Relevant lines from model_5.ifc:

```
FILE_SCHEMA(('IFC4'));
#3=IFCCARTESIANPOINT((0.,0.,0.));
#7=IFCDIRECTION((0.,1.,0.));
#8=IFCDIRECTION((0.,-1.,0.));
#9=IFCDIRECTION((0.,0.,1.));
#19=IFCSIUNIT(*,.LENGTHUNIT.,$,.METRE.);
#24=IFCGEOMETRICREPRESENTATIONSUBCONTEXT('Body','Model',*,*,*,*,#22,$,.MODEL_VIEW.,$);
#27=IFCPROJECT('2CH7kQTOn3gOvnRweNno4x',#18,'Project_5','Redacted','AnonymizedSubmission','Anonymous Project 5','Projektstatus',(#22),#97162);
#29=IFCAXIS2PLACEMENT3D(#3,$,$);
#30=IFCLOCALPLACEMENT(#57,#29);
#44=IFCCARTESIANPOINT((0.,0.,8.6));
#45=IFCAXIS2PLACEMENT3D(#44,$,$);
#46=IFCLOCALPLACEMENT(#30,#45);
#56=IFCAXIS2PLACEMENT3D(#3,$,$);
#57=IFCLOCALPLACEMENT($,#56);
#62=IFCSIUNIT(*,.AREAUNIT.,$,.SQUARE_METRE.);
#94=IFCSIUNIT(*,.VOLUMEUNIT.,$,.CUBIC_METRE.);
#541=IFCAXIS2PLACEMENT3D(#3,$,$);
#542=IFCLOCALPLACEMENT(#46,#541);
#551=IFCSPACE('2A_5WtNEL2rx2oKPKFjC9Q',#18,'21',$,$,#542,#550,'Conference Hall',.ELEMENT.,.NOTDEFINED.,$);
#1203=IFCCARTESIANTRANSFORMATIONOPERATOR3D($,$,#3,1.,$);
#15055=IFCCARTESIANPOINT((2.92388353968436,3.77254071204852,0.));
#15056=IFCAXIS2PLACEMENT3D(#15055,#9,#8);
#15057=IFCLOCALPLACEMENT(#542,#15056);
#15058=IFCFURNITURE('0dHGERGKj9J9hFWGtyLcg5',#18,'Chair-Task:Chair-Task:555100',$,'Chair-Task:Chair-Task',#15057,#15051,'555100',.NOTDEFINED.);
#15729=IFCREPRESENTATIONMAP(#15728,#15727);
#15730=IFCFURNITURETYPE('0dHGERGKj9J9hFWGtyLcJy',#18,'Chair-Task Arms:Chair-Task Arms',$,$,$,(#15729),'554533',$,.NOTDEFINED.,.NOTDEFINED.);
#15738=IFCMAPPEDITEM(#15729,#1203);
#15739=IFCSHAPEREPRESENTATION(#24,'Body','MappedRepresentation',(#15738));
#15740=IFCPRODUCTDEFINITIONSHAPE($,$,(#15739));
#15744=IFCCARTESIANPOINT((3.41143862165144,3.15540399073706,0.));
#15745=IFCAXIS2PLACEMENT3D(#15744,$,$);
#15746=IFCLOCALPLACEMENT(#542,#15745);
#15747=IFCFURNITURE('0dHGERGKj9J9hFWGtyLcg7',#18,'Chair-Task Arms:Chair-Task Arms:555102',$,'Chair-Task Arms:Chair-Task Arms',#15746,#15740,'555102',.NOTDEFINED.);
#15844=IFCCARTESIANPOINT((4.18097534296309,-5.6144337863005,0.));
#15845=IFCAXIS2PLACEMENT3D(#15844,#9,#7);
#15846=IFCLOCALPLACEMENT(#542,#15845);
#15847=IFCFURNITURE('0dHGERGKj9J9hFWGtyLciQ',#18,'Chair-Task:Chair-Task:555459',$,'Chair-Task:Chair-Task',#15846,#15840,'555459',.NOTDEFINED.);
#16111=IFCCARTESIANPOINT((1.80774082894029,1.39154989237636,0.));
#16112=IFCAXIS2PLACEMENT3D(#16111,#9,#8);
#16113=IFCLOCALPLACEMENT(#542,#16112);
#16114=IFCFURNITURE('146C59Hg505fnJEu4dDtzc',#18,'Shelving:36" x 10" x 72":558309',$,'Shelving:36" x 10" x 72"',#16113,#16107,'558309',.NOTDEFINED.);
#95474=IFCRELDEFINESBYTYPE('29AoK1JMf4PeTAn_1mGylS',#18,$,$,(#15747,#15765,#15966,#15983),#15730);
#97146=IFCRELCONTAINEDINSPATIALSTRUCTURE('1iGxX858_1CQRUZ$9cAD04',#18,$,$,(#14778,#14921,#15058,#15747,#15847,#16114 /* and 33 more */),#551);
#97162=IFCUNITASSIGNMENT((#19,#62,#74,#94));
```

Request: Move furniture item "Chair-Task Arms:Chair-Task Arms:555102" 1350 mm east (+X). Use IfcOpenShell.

```python
import ifcopenshell
import ifcopenshell.api.geometry
import ifcopenshell.util.placement
import ifcopenshell.util.unit

model = ifcopenshell.open("model_5.ifc")
unit_scale = ifcopenshell.util.unit.calculate_unit_scale(model)

item = model.by_guid("0dHGERGKj9J9hFWGtyLcg7")
matrix = ifcopenshell.util.placement.get_local_placement(item.ObjectPlacement)
matrix[0, 3] += 1.35 / unit_scale
ifcopenshell.api.geometry.edit_object_placement(model, product=item, matrix=matrix, is_si=False)

print(ifcopenshell.util.placement.get_local_placement(item.ObjectPlacement).round(3) + 0.0)

model.write("model_5_updated.ifc")
```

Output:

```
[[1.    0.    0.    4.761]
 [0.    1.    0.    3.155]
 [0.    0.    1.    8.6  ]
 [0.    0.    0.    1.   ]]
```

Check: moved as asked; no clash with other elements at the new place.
